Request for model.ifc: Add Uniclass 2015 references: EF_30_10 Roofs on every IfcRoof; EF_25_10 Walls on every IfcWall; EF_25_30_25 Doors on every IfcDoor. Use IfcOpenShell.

First a look at what the model holds.

```python
import ifcopenshell

model = ifcopenshell.open("model.ifc")
print(model.schema)
print("classifications:", [c.Name for c in model.by_type("IfcClassification")])
for ifc_class in ("IfcDoor", "IfcRoof", "IfcStair", "IfcWall", "IfcWindow"):
    print(ifc_class, len(model.by_type(ifc_class)))
```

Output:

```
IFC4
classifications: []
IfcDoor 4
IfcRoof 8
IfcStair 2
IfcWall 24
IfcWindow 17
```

```python
import ifcopenshell
import ifcopenshell.api.classification

model = ifcopenshell.open("model.ifc")

system = ifcopenshell.api.classification.add_classification(model, classification="Uniclass 2015")

codes = {
    "IfcRoof": ("EF_30_10", "Roofs"),
    "IfcWall": ("EF_25_10", "Walls"),
    "IfcDoor": ("EF_25_30_25", "Doors"),
}
for ifc_class, (code, name) in codes.items():
    products = model.by_type(ifc_class)
    ifcopenshell.api.classification.add_reference(
        model, products=products, classification=system, identification=code, name=name
    )
    print(code, len(products))

model.write("model_updated.ifc")
```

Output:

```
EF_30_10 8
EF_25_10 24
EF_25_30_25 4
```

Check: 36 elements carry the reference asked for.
